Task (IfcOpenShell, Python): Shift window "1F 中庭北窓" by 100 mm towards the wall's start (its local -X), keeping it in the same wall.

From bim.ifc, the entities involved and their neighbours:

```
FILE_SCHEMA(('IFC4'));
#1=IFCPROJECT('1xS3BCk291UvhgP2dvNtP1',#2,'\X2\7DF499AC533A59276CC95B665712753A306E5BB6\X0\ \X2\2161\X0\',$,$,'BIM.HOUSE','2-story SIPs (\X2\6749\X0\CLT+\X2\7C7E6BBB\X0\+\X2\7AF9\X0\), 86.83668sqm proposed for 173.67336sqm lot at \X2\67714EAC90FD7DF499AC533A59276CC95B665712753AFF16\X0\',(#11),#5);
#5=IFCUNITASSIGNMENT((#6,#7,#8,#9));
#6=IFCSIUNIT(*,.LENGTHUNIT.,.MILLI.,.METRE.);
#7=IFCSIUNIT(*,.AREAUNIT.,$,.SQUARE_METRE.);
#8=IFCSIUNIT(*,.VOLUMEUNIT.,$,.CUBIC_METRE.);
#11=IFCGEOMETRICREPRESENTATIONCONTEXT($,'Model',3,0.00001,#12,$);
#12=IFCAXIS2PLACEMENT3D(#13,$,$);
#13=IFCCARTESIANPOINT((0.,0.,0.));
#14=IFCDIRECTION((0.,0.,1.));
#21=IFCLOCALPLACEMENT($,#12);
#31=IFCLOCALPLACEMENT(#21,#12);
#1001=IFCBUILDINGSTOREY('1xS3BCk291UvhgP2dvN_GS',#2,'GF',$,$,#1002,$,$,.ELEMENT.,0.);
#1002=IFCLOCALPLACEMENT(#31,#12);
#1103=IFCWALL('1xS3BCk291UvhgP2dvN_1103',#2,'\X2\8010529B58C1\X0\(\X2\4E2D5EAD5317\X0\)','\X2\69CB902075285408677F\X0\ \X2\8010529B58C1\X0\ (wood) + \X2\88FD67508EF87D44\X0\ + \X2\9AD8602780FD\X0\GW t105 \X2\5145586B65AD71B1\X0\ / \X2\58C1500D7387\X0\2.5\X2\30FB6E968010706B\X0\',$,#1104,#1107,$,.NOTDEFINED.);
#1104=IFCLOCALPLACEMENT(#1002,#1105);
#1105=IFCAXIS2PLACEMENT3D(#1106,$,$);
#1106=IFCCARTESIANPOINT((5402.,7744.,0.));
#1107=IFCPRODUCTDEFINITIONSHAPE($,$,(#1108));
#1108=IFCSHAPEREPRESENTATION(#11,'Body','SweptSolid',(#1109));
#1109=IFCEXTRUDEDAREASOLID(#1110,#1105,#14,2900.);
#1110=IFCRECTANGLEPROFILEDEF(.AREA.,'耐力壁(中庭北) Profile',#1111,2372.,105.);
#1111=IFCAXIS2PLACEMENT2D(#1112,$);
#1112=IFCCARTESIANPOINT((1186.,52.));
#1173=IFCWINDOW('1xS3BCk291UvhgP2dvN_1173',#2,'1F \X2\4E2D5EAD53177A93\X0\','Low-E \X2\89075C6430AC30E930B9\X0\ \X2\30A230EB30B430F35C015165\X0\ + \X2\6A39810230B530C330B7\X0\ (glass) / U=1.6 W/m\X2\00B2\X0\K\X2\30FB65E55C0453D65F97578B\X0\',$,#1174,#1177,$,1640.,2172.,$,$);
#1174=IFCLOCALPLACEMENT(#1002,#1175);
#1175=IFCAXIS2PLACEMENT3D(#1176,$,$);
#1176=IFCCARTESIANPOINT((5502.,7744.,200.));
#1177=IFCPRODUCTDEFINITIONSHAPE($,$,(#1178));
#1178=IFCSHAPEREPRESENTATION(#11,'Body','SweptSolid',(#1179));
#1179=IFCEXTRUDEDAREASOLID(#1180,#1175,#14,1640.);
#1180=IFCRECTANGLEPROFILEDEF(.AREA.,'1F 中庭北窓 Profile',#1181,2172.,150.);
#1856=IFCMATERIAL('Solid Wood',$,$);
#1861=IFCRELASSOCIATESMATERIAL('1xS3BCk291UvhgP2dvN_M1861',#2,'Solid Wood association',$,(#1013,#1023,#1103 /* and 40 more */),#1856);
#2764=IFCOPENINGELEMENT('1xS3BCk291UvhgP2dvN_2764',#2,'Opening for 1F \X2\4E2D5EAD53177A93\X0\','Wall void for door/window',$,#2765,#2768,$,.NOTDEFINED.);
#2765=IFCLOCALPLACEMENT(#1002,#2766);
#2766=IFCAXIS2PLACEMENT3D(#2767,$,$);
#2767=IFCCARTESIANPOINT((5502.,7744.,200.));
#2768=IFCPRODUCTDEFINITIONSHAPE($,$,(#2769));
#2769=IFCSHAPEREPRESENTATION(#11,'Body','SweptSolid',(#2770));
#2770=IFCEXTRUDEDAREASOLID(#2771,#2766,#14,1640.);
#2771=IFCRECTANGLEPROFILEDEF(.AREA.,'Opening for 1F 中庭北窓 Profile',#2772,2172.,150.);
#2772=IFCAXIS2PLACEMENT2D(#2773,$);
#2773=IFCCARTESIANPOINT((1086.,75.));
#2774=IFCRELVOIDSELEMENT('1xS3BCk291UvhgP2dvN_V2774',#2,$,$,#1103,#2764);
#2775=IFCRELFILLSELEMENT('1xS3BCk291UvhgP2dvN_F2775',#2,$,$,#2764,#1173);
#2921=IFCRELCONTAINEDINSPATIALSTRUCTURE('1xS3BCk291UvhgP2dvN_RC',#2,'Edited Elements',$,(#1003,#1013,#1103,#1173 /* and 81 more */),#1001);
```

```python
import ifcopenshell
import ifcopenshell.api.geometry
import ifcopenshell.util.placement
import ifcopenshell.util.unit

model = ifcopenshell.open("bim.ifc")
unit_scale = ifcopenshell.util.unit.calculate_unit_scale(model)

window = model.by_guid("1xS3BCk291UvhgP2dvN_1173")
opening = window.FillsVoids[0].RelatingOpeningElement
wall = opening.VoidsElements[0].RelatingBuildingElement

wall_matrix = ifcopenshell.util.placement.get_local_placement(wall.ObjectPlacement)
shift = wall_matrix[:3, 0] * -0.1 / unit_scale
before = ifcopenshell.util.placement.get_local_placement(window.ObjectPlacement)[:3, 3].copy()

# The window is not placed relative to its opening, so move both.
for product in (opening, window):
    matrix = ifcopenshell.util.placement.get_local_placement(product.ObjectPlacement)
    matrix[:3, 3] += shift
    ifcopenshell.api.geometry.edit_object_placement(model, product=product, matrix=matrix, is_si=False)

after = ifcopenshell.util.placement.get_local_placement(window.ObjectPlacement)[:3, 3]
print("window moved by", (after - before).round(3) + 0.0)

model.write("bim-out.ifc")
```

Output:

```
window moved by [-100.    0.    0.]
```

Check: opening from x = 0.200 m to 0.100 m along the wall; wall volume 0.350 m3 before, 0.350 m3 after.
